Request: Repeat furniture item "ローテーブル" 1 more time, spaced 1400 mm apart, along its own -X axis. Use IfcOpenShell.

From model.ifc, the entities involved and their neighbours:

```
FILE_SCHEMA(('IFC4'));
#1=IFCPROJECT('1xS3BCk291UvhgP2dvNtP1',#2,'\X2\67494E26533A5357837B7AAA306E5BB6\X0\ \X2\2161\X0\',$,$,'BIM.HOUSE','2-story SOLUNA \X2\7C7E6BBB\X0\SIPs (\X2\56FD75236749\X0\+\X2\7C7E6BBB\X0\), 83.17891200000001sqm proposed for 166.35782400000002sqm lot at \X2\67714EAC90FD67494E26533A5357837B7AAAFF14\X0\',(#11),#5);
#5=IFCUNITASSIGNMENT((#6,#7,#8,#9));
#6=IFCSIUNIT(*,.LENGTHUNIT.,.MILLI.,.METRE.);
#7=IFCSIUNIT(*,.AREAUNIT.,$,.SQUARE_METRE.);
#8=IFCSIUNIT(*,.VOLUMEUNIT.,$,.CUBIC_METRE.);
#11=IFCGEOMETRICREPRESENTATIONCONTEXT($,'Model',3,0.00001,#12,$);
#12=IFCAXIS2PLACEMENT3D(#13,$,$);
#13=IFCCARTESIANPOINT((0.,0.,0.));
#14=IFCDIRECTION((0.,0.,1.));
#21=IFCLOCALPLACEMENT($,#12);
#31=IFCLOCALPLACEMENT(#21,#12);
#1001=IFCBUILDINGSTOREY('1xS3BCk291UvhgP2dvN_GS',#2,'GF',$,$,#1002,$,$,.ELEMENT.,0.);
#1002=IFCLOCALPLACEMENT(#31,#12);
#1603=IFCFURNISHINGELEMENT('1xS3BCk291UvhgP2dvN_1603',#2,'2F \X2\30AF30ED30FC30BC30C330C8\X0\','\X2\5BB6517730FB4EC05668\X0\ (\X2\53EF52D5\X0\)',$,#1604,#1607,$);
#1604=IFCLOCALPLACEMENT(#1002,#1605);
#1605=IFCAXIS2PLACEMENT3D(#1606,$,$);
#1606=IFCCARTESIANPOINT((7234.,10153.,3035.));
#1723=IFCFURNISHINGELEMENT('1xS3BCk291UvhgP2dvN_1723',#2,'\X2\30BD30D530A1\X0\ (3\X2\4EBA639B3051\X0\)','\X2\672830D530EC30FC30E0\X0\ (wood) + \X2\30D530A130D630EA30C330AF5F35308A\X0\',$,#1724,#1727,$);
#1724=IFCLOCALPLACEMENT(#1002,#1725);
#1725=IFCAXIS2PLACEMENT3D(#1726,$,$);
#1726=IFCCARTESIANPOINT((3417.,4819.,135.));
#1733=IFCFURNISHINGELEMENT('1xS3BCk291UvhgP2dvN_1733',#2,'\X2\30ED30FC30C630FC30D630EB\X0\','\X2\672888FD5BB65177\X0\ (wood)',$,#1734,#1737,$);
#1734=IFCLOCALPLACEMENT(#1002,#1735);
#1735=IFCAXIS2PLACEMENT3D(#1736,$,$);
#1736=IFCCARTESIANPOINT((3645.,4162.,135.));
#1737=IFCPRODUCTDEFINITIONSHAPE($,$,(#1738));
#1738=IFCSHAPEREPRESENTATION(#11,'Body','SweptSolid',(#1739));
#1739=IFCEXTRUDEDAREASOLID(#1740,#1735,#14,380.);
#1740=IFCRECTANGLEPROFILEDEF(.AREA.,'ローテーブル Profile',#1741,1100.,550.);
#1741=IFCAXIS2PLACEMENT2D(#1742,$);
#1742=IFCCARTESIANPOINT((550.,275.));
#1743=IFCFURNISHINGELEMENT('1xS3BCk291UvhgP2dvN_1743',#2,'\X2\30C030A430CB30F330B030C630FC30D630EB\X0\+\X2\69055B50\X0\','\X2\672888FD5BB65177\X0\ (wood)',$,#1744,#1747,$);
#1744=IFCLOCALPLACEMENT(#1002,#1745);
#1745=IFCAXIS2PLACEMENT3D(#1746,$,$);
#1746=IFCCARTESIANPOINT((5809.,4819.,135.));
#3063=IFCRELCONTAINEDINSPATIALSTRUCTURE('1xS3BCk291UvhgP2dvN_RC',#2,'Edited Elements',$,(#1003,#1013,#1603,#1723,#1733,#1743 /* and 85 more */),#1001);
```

```python
import ifcopenshell
import ifcopenshell.api.geometry
import ifcopenshell.api.root
import ifcopenshell.util.element
import ifcopenshell.util.placement
import ifcopenshell.util.unit

model = ifcopenshell.open("model.ifc")
unit_scale = ifcopenshell.util.unit.calculate_unit_scale(model)


def reuse_history(source, copy):
    """copy_class also copies each property set's owner history, people and application; keep the originals."""
    for rel in copy.IsDefinedBy:
        if rel.is_a("IfcRelDefinesByProperties") and (history := rel.RelatingPropertyDefinition.OwnerHistory):
            rel.RelatingPropertyDefinition.OwnerHistory = source.OwnerHistory
            ifcopenshell.util.element.remove_deep2(model, history)


source = model.by_id(1733)
base = ifcopenshell.util.placement.get_local_placement(source.ObjectPlacement)
step = -base[:3, 0] * 1.4 / unit_scale

for i in range(1, 2):
    copy = ifcopenshell.api.root.copy_class(model, product=source)
    copy.Representation = ifcopenshell.util.element.copy_deep(
        model, source.Representation, exclude=["IfcGeometricRepresentationContext", "IfcRepresentationMap"]
    )
    reuse_history(source, copy)
    matrix = base.copy()
    matrix[:3, 3] += i * step
    print("added at", matrix[:3, 3].round(3) + 0.0)
    ifcopenshell.api.geometry.edit_object_placement(model, product=copy, matrix=matrix, is_si=False)

model.write("model_edited.ifc")
```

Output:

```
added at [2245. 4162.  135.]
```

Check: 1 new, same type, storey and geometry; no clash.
